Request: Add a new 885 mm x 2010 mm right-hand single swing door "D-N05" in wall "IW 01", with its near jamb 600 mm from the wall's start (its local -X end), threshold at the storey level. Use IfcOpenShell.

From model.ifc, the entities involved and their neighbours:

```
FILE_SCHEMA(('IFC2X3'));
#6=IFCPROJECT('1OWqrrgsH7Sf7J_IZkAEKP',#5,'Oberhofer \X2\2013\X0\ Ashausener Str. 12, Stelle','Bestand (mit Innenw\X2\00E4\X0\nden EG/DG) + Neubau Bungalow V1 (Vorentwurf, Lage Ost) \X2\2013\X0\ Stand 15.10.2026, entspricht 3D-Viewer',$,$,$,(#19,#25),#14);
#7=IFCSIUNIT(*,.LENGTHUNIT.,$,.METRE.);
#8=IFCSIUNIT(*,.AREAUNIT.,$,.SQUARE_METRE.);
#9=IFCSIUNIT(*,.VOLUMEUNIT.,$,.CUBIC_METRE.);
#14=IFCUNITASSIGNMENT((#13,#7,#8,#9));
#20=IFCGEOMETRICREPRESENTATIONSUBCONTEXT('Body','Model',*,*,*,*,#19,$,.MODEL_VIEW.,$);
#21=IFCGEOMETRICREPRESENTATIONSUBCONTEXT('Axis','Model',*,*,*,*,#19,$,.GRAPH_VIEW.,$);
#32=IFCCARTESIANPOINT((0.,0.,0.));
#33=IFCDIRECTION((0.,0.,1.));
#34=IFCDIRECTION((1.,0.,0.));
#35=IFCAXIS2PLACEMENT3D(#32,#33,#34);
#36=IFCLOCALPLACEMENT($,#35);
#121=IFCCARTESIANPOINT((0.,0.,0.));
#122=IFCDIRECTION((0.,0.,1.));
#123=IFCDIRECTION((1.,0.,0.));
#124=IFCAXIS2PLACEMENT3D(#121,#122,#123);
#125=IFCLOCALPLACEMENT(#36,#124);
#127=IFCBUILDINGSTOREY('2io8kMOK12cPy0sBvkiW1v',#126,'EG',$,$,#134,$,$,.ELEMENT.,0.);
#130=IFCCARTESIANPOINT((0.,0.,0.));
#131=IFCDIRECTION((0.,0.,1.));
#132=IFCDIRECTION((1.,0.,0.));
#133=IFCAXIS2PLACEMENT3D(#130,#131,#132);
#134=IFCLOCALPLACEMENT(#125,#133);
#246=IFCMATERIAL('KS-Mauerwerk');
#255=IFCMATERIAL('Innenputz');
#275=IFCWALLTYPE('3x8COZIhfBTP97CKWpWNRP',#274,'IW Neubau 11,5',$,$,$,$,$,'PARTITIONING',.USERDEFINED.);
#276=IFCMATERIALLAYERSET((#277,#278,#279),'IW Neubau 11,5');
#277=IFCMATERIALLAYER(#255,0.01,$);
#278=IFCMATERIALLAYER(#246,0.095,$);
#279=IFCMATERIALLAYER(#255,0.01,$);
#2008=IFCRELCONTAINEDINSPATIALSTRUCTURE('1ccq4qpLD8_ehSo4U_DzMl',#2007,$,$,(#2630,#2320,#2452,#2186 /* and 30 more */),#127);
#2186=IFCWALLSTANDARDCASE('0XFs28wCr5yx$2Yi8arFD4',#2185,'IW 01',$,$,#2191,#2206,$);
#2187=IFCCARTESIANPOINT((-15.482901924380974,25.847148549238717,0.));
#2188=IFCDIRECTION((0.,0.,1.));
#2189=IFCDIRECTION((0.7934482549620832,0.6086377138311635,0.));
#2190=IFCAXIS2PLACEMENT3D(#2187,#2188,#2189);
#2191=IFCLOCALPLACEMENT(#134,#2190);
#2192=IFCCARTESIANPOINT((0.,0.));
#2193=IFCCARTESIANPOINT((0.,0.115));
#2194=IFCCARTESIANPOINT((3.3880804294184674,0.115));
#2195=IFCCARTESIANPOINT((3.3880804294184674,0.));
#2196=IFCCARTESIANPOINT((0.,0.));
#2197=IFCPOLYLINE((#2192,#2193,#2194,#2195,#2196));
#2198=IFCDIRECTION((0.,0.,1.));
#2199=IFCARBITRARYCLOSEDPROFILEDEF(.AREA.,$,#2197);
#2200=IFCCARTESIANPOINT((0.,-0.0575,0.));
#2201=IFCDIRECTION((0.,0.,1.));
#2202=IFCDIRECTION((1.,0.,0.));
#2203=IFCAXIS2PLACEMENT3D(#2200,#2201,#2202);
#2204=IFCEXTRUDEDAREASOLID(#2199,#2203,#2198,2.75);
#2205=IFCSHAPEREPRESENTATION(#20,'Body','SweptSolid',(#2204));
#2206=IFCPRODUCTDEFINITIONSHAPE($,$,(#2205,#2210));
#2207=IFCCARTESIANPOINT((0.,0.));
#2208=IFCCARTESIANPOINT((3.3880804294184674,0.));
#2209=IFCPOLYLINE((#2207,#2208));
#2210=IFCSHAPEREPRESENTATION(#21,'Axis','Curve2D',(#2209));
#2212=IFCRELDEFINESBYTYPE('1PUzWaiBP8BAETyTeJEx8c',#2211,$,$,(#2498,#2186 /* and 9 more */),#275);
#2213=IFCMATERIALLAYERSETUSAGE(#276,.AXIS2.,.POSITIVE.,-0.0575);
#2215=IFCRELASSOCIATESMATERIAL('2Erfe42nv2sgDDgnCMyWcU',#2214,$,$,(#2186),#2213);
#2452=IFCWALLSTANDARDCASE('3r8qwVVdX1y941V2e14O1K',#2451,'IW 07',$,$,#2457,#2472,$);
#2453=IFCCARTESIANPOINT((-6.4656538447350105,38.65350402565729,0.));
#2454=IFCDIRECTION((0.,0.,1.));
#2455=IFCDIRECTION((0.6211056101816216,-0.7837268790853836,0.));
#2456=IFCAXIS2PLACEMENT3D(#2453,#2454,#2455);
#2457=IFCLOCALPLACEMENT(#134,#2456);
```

```python
import numpy as np
import ifcopenshell
import ifcopenshell.api.feature
import ifcopenshell.api.geometry
import ifcopenshell.api.root
import ifcopenshell.api.spatial
import ifcopenshell.api.type
import ifcopenshell.geom
import ifcopenshell.util.element
import ifcopenshell.util.placement
import ifcopenshell.util.representation
import ifcopenshell.util.shape
import ifcopenshell.util.unit

model = ifcopenshell.open("model.ifc")
unit_scale = ifcopenshell.util.unit.calculate_unit_scale(model)
settings = ifcopenshell.geom.settings()


def volume(element):
    """Net volume in cubic metres, openings subtracted."""
    shape = ifcopenshell.geom.create_shape(settings, element)
    return ifcopenshell.util.shape.get_volume(shape.geometry)


wall = model.by_guid("0XFs28wCr5yx$2Yi8arFD4")
storey = ifcopenshell.util.element.get_container(wall, ifc_class="IfcBuildingStorey")
context = ifcopenshell.util.representation.get_context(model, "Model", "Body", "MODEL_VIEW")
before = volume(wall)

width, height, from_end, sill = 0.885, 2.01, 0.6, 0.0  # metres

# The wall runs along its own X axis, and the end named is its -X end.
wall_shape = ifcopenshell.geom.create_shape(settings, wall)
x, y, z = ifcopenshell.util.shape.get_vertices(wall_shape.geometry).T
start = x.min() + from_end
face, thickness = float(y.min()), float(y.max() - y.min())
wall_matrix = ifcopenshell.util.placement.get_local_placement(wall.ObjectPlacement)
level = ifcopenshell.util.placement.get_local_placement(storey.ObjectPlacement)[2, 3]


def in_wall(x, y):
    """Placement at x, y metres in the wall's axes, at sill height."""
    matrix = wall_matrix.copy()
    matrix[:, 3] = wall_matrix @ np.array([x / unit_scale, y / unit_scale, 0.0, 1.0])
    matrix[2, 3] = level + sill / unit_scale
    return matrix


# Opening: a box that overshoots both wall faces by 50 mm.
opening = ifcopenshell.api.root.create_entity(model, ifc_class="IfcOpeningElement")
box = ifcopenshell.api.geometry.add_wall_representation(
    model, context=context, length=width, height=height, thickness=thickness + 0.1
)
ifcopenshell.api.geometry.assign_representation(model, product=opening, representation=box)
ifcopenshell.api.geometry.edit_object_placement(model, product=opening, matrix=in_wall(start, face - 0.05), is_si=False)
ifcopenshell.api.feature.add_feature(model, feature=opening, element=wall)

door = ifcopenshell.api.root.create_entity(model, ifc_class="IfcDoor", name="D-N05")
door.OverallWidth, door.OverallHeight = width / unit_scale, height / unit_scale
body = ifcopenshell.api.geometry.add_door_representation(
    model,
    context=context,
    overall_width=door.OverallWidth,
    overall_height=door.OverallHeight,
    operation_type="SINGLE_SWING_RIGHT",
    lining_properties={"LiningDepth": thickness / unit_scale, "ThresholdDepth": thickness / unit_scale},
)
ifcopenshell.api.geometry.assign_representation(model, product=door, representation=body)
ifcopenshell.api.spatial.assign_container(model, products=[door], relating_structure=storey)
fills = ifcopenshell.api.feature.add_filling(model, opening=opening, element=door)
fills.OwnerHistory = door.OwnerHistory  # required in IFC2X3

# IFC2X3 keeps the operation on the door style.
style = ifcopenshell.api.root.create_entity(model, ifc_class="IfcDoorStyle", name="D-N05")
style.OperationType, style.ConstructionType = "SINGLE_SWING_RIGHT", "NOTDEFINED"
style.ParameterTakesPrecedence = style.Sizeable = False
ifcopenshell.api.type.assign_type(model, related_objects=[door], relating_type=style)

# The lining spans the wall, so the door starts at the wall face.
ifcopenshell.api.geometry.edit_object_placement(model, product=door, matrix=in_wall(start, face), is_si=False)

after = volume(wall)

print(f"wall volume {before:.3f} -> {after:.3f} m3")

model.write("model_rev.ifc")
```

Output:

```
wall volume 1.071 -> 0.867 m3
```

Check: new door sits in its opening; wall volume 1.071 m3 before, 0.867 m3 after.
